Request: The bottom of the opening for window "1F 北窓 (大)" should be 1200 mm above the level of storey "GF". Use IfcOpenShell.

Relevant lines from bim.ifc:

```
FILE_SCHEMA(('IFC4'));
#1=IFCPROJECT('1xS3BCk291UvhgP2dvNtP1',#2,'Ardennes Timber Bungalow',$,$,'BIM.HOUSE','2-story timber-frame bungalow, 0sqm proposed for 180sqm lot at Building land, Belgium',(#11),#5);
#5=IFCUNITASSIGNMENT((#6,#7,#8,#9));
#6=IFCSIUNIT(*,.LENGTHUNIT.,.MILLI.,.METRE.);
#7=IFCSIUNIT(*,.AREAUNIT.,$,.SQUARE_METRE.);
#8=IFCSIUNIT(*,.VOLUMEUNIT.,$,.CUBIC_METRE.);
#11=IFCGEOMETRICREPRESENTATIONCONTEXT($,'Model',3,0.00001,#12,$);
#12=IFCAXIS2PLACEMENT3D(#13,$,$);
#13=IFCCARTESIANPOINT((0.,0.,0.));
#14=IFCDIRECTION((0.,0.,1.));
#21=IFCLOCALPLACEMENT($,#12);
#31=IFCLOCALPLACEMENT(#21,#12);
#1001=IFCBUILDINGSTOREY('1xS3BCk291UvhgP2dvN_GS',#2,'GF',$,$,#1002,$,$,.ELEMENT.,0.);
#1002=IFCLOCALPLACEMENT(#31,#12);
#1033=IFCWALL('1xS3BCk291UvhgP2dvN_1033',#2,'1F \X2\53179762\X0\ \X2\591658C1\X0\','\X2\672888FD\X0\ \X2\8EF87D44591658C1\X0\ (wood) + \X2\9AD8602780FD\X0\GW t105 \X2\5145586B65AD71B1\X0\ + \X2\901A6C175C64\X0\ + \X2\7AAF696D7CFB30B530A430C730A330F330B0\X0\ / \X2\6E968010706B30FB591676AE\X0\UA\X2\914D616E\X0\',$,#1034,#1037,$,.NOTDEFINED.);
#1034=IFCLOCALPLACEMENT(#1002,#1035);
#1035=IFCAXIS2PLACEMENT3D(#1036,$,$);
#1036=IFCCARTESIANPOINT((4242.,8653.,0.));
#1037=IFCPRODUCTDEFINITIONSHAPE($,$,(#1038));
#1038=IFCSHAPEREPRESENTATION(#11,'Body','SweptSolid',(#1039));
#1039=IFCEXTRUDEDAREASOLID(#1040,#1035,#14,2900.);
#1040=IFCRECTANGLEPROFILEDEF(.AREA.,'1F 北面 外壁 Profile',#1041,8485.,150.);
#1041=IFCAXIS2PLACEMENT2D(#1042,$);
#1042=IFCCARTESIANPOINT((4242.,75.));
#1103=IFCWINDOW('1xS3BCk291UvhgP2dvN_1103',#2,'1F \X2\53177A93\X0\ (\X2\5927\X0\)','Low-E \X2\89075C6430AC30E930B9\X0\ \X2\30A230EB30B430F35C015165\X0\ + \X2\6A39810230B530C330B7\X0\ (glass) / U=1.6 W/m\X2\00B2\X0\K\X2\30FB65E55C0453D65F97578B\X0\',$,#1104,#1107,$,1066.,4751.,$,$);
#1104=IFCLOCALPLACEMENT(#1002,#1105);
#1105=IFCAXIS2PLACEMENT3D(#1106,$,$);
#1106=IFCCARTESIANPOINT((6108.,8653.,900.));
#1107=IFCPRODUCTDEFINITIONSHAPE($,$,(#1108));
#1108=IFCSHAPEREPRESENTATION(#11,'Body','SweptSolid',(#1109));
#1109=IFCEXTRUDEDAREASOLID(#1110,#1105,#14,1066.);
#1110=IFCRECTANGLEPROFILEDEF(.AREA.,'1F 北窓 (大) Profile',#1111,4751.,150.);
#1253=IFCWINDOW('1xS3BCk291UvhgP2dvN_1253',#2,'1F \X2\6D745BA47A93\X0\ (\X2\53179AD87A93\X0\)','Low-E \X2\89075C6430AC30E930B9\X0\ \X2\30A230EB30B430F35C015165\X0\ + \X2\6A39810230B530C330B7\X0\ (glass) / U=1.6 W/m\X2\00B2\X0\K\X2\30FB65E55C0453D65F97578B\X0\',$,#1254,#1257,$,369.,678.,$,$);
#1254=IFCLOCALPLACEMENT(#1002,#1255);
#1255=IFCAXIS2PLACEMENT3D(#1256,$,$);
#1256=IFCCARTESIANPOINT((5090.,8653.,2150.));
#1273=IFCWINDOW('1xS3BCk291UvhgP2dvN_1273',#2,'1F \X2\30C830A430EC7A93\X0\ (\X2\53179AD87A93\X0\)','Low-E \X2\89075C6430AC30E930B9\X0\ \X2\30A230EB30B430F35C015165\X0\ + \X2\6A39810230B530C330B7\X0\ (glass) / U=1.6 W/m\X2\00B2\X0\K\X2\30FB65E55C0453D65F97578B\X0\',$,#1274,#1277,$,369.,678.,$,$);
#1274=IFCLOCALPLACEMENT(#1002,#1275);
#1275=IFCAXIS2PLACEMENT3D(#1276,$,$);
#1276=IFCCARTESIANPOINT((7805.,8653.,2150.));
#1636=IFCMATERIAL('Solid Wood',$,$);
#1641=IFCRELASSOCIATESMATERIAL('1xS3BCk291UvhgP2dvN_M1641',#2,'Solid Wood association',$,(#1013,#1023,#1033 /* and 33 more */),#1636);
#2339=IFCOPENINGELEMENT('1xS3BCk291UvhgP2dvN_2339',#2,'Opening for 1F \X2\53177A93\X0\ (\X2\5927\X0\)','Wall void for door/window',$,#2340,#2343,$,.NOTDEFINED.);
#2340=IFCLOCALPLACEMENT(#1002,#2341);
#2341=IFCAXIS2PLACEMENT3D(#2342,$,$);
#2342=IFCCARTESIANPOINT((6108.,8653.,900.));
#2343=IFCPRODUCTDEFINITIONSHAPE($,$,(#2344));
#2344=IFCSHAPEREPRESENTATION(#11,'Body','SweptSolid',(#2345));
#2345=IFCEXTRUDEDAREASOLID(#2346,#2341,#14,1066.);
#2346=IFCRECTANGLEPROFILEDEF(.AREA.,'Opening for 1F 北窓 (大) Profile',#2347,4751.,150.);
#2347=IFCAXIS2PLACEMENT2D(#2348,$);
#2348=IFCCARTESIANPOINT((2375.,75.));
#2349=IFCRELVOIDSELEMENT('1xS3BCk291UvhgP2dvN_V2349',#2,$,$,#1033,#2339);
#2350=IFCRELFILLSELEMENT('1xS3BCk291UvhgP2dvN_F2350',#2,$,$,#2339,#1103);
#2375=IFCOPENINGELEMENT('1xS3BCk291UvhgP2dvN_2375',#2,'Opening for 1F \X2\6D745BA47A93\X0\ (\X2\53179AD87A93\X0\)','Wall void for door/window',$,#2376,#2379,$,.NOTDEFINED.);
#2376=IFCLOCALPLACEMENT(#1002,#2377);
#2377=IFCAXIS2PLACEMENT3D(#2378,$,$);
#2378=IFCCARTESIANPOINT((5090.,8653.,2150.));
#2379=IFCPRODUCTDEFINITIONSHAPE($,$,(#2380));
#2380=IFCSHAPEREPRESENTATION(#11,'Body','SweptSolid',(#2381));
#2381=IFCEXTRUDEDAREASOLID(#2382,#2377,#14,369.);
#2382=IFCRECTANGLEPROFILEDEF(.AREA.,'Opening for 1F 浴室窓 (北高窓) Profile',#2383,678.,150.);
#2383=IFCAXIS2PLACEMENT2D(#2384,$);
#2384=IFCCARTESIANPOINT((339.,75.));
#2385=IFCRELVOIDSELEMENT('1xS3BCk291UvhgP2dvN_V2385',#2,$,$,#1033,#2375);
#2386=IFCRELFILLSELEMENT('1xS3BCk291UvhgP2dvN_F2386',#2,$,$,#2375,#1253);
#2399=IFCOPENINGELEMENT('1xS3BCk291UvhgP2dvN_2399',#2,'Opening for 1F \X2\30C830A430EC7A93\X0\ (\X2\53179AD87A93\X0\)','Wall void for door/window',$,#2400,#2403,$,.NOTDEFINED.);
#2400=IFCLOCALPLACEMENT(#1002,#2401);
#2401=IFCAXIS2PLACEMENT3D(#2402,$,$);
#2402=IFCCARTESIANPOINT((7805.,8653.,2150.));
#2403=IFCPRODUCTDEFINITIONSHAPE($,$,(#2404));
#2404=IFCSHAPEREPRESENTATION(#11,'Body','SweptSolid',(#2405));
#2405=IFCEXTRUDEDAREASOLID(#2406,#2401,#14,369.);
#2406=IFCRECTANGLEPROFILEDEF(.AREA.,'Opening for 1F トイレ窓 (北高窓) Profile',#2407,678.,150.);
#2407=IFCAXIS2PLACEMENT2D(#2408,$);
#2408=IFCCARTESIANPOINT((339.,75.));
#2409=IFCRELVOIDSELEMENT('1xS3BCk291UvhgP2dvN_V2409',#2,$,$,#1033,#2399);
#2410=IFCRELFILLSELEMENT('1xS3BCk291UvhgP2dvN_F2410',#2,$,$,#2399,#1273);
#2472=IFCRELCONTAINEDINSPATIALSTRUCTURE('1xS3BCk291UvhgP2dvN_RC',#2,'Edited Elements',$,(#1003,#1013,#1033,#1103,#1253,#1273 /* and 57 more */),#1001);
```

```python
import numpy as np
import ifcopenshell
import ifcopenshell.api.geometry
import ifcopenshell.geom
import ifcopenshell.util.element
import ifcopenshell.util.placement
import ifcopenshell.util.shape
import ifcopenshell.util.unit

model = ifcopenshell.open("bim.ifc")
unit_scale = ifcopenshell.util.unit.calculate_unit_scale(model)

window = model.by_guid("1xS3BCk291UvhgP2dvN_1103")
opening = window.FillsVoids[0].RelatingOpeningElement
storey = ifcopenshell.util.element.get_container(window, ifc_class="IfcBuildingStorey")
level = ifcopenshell.util.placement.get_local_placement(storey.ObjectPlacement)[2, 3]

# The opening's origin need not be at the sill, so measure its lowest point.
shape = ifcopenshell.geom.create_shape(ifcopenshell.geom.settings(), opening)
bottom = ifcopenshell.util.shape.get_shape_bottom_elevation(shape, shape.geometry) / unit_scale
dz = level + 1200.0 - bottom

shift = np.array([0.0, 0.0, dz])
# The window is not placed relative to its opening, so move both.
for product in (opening, window):
    matrix = ifcopenshell.util.placement.get_local_placement(product.ObjectPlacement)
    matrix[:3, 3] += shift
    ifcopenshell.api.geometry.edit_object_placement(model, product=product, matrix=matrix, is_si=False)

print(f"moved by {dz * unit_scale:+.3f} m")

model.write("bim_v2.ifc")
```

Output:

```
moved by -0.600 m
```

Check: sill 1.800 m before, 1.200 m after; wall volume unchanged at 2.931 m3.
